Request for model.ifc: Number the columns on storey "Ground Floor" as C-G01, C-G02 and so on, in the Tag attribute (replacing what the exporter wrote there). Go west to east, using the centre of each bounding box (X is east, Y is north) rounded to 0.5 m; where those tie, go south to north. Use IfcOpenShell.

First a look at what the model holds.

```python
import ifcopenshell
import ifcopenshell.util.element
import ifcopenshell.util.placement

model = ifcopenshell.open("model.ifc")
print(model.schema)
storey = next(s for s in model.by_type("IfcBuildingStorey") if s.Name == "Ground Floor")
columns = [e for e in ifcopenshell.util.element.get_decomposition(storey) if e.is_a("IfcColumn")]
for e in sorted(columns, key=lambda e: e.id()):
    origin = ifcopenshell.util.placement.get_local_placement(e.ObjectPlacement)[:3, 3]
    print(e.id(), e.Tag, e.Name, origin.round(2) + 0.0, sep=" | ")
```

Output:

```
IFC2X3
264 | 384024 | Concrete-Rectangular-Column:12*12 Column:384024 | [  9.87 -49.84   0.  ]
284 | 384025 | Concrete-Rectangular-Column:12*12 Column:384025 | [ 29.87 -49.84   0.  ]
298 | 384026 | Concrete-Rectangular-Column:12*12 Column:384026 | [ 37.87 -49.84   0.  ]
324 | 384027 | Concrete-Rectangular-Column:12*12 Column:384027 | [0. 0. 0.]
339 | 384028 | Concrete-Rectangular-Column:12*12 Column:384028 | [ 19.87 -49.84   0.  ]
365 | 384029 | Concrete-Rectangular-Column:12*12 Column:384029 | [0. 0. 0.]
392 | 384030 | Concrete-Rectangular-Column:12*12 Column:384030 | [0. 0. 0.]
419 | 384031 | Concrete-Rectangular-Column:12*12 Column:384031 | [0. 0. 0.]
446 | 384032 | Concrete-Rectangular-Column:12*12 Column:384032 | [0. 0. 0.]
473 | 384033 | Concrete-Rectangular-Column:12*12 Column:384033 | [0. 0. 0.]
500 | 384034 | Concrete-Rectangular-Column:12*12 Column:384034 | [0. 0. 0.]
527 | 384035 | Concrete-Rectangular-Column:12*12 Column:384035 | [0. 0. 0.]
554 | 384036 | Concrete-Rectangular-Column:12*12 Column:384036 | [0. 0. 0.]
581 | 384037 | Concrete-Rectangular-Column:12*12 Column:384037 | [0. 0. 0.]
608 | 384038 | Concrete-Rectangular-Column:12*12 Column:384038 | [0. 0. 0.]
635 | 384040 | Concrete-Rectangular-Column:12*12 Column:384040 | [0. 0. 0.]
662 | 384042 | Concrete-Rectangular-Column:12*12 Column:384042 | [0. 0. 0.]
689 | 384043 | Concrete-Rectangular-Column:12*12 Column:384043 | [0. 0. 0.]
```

```python
import ifcopenshell
import ifcopenshell.geom
import ifcopenshell.util.element
import ifcopenshell.util.shape

model = ifcopenshell.open("model.ifc")
settings = ifcopenshell.geom.settings()
settings.set("use-world-coords", True)


def centre(element):
    shape = ifcopenshell.geom.create_shape(settings, element)
    return ifcopenshell.util.shape.get_bbox_centroid(shape.geometry)


storey = next(s for s in model.by_type("IfcBuildingStorey") if s.Name == "Ground Floor")
columns = [e for e in ifcopenshell.util.element.get_decomposition(storey) if e.is_a("IfcColumn")]

# Insertion points can sit at a corner or the storey origin, so sort by the geometry (in metres).
centres = {e: centre(e) for e in columns}
columns.sort(key=lambda e: (round(centres[e][0] / 0.5), centres[e][1]))

for i, e in enumerate(columns, start=1):
    number = f"C-G{i:02d}"
    e.Tag = number
    print(e.id(), number)

model.write("model_updated.ifc")
```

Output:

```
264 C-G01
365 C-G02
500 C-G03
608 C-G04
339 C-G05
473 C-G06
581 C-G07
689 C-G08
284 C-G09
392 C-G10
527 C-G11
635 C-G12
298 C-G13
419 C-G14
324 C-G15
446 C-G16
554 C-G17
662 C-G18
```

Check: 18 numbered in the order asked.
